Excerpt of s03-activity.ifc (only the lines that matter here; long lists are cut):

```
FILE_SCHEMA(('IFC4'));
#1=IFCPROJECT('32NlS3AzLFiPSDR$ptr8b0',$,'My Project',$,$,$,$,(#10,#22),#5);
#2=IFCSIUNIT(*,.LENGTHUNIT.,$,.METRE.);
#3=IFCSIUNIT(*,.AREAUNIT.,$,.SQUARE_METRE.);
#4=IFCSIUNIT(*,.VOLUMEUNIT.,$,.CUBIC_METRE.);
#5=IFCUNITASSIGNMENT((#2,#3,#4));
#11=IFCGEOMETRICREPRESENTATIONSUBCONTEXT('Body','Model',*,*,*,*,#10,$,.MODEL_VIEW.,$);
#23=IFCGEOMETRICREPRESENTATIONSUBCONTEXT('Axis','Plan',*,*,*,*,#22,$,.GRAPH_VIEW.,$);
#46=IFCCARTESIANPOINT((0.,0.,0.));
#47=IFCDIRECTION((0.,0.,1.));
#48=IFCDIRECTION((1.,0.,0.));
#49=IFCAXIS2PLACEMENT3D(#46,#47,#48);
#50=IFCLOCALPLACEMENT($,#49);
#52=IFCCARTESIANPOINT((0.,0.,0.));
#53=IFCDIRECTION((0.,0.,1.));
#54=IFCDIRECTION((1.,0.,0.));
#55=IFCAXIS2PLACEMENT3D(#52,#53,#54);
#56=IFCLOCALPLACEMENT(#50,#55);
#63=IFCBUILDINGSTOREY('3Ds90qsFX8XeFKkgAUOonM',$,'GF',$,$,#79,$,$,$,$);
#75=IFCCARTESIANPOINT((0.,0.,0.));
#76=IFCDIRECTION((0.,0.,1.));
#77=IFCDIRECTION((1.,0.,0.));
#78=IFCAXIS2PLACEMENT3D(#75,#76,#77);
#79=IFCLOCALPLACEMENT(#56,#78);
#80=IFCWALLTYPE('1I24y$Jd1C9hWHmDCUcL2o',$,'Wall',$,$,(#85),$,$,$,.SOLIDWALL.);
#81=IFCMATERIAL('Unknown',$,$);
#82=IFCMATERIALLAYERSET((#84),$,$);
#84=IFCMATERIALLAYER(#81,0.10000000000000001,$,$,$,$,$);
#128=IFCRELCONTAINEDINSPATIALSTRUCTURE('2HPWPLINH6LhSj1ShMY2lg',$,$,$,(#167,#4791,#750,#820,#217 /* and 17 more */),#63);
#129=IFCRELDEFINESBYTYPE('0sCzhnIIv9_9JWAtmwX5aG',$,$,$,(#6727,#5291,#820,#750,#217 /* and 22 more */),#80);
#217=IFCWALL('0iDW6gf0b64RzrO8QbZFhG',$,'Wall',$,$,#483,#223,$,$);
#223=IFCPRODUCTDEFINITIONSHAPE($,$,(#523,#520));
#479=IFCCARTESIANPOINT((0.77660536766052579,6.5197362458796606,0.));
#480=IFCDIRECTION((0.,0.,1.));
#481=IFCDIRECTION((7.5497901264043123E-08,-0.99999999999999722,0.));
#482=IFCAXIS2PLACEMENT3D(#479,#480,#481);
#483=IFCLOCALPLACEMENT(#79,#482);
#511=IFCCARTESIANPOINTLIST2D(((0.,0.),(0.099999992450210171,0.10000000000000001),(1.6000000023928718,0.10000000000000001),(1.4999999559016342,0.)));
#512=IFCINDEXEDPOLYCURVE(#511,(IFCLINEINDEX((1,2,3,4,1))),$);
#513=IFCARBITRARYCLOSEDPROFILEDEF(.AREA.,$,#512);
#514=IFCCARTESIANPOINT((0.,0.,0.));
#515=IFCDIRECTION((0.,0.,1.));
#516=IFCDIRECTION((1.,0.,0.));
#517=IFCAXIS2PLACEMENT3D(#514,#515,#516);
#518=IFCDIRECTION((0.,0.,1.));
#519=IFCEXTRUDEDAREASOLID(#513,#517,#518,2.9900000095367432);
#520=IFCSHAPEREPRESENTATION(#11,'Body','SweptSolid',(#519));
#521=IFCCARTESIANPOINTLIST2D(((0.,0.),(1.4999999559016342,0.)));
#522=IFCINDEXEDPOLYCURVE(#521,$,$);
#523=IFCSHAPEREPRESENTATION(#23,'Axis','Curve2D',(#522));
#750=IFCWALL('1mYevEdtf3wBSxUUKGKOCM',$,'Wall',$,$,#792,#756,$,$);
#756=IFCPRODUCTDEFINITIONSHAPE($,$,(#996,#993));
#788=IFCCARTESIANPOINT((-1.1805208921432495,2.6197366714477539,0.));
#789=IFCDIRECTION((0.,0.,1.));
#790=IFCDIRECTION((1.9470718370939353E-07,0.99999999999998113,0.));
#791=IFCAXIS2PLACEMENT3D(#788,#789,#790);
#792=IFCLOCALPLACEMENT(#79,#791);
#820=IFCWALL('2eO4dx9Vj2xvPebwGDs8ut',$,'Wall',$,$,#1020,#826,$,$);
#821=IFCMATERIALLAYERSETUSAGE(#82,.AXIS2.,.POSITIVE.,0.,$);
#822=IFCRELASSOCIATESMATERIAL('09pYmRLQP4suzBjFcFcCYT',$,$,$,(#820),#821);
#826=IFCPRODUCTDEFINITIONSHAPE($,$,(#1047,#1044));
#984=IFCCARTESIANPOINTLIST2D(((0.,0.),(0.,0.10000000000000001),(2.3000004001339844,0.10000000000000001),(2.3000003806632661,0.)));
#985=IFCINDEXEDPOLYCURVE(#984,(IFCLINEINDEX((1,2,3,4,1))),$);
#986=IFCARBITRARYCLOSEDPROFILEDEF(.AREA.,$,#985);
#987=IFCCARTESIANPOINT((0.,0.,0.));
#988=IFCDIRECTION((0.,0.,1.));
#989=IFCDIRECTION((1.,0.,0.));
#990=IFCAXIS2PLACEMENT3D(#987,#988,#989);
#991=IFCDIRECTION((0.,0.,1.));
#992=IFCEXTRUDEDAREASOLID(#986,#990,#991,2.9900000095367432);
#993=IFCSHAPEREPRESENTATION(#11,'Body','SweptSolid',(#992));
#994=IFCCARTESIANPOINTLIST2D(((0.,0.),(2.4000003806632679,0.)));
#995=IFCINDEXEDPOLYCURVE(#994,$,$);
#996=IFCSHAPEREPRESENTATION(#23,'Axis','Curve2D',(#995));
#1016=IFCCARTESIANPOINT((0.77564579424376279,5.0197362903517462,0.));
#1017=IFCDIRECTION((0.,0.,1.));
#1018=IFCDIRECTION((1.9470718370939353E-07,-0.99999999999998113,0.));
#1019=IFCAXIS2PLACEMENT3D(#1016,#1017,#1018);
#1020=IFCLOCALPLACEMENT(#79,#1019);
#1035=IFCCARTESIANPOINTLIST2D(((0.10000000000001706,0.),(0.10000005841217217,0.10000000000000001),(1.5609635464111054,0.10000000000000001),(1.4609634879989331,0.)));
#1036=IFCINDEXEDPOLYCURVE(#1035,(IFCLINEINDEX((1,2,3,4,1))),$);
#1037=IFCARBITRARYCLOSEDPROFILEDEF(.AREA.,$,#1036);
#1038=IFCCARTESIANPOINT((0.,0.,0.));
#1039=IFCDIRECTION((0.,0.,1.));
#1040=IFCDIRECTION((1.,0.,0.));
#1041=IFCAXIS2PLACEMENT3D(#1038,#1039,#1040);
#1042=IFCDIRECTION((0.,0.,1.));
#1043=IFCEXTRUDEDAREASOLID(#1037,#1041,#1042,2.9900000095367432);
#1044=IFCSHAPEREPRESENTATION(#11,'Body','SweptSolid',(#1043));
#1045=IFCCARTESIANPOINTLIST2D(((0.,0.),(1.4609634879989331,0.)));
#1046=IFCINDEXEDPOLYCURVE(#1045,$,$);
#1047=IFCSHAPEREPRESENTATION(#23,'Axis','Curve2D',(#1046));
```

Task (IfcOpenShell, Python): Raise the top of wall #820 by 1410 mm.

```python
import ifcopenshell
import ifcopenshell.geom
import ifcopenshell.util.representation
import ifcopenshell.util.shape
import ifcopenshell.util.unit

model = ifcopenshell.open("s03-activity.ifc")
unit_scale = ifcopenshell.util.unit.calculate_unit_scale(model)
settings = ifcopenshell.geom.settings()


def volume(element):
    """Net volume in cubic metres, openings subtracted."""
    shape = ifcopenshell.geom.create_shape(settings, element)
    return ifcopenshell.util.shape.get_volume(shape.geometry)


wall = model.by_id(820)
before = volume(wall)

body = ifcopenshell.util.representation.get_representation(wall, "Model", "Body")
solid = body.Items[0]
old_height = solid.Depth
solid.Depth += 1.41 / unit_scale
after = volume(wall)

print(f"height {old_height:g} -> {solid.Depth:g}, volume {before:.3f} -> {after:.3f} m3")

model.write("s03-activity_rev.ifc")
```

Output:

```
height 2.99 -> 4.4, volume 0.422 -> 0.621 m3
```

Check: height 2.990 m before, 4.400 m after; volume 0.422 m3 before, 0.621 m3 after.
